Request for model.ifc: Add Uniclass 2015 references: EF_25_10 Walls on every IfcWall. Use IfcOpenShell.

First a look at what the model holds.

```python
import ifcopenshell

model = ifcopenshell.open("model.ifc")
print(model.schema)
print("classifications:", [c.Name for c in model.by_type("IfcClassification")])
for ifc_class in ("IfcDoor", "IfcRoof", "IfcStair", "IfcWall", "IfcWindow"):
    print(ifc_class, len(model.by_type(ifc_class)))
```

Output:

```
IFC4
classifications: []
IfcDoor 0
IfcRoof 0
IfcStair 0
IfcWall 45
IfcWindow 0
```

```python
import ifcopenshell
import ifcopenshell.api.classification

model = ifcopenshell.open("model.ifc")

system = ifcopenshell.api.classification.add_classification(model, classification="Uniclass 2015")

codes = {
    "IfcWall": ("EF_25_10", "Walls"),
}
for ifc_class, (code, name) in codes.items():
    products = model.by_type(ifc_class)
    ifcopenshell.api.classification.add_reference(
        model, products=products, classification=system, identification=code, name=name
    )
    print(code, len(products))

model.write("model_rev.ifc")
```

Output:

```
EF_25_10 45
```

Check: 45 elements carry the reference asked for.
